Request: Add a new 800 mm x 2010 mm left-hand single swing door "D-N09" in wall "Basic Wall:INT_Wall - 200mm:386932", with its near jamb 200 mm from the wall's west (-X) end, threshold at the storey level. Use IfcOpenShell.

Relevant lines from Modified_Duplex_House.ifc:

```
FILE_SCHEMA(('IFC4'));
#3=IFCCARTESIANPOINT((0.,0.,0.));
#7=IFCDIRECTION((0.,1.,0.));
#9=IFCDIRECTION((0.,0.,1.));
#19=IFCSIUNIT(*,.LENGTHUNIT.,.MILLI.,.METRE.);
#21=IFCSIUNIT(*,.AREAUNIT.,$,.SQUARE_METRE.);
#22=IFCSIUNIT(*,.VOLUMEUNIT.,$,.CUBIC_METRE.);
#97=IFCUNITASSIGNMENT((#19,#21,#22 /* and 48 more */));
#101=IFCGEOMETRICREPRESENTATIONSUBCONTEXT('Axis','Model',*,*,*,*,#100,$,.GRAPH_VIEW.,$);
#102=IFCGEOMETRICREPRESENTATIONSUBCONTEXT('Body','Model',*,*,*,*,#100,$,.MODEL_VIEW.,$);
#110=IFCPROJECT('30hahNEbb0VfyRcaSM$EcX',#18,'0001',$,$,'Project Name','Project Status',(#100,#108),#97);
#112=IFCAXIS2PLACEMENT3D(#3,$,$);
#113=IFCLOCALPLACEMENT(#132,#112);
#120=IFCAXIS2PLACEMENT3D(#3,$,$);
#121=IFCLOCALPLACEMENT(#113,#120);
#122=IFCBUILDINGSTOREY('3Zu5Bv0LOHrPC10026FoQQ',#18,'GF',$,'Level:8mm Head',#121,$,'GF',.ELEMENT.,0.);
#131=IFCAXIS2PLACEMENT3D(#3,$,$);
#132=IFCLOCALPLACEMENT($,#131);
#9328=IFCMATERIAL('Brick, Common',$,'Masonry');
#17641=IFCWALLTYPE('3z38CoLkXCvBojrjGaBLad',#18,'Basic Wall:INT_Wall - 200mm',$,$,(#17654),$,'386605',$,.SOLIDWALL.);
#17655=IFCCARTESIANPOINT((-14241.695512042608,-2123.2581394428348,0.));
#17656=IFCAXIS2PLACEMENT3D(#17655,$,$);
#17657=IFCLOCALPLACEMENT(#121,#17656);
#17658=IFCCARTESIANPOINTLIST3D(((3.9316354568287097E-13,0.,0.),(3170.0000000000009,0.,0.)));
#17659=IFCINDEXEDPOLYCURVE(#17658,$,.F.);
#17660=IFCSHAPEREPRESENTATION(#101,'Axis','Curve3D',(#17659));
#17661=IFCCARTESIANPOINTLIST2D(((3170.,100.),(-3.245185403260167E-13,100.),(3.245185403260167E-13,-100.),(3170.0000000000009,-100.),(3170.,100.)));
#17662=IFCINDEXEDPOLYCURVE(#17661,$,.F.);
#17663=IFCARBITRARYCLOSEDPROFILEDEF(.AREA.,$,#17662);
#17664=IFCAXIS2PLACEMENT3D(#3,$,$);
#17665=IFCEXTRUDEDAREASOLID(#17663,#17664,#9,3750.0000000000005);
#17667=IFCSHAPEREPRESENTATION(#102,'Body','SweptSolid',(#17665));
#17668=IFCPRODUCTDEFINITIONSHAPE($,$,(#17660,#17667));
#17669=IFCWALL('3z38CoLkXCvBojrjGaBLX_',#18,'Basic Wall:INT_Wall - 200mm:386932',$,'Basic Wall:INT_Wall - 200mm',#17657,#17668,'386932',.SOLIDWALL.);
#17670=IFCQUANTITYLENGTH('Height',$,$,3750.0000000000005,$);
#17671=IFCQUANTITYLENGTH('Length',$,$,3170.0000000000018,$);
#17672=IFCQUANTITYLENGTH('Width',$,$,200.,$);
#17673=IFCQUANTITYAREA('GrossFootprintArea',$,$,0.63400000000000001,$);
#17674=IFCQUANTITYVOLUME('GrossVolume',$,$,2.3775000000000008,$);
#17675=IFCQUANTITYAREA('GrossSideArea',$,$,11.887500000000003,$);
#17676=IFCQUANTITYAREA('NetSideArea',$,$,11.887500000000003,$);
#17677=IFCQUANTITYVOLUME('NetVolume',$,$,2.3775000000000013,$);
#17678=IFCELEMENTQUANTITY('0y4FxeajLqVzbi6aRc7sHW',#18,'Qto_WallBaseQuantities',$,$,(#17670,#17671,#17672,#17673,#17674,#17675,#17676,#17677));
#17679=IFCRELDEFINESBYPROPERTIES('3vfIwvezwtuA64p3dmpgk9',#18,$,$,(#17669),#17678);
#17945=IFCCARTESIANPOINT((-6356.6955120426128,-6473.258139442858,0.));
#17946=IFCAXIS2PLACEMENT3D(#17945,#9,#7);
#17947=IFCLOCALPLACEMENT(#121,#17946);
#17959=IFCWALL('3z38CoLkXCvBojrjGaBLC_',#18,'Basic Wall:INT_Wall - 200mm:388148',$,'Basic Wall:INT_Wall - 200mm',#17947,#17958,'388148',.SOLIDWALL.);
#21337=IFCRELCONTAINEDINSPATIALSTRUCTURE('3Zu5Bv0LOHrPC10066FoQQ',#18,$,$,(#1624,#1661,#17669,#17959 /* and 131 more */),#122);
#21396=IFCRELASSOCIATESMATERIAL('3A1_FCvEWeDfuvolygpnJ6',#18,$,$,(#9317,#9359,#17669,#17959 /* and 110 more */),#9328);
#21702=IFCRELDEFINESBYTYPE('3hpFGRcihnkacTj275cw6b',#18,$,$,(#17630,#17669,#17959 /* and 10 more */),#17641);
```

```python
import numpy as np
import ifcopenshell
import ifcopenshell.api.feature
import ifcopenshell.api.geometry
import ifcopenshell.api.pset
import ifcopenshell.api.root
import ifcopenshell.api.spatial
import ifcopenshell.geom
import ifcopenshell.util.element
import ifcopenshell.util.placement
import ifcopenshell.util.representation
import ifcopenshell.util.shape
import ifcopenshell.util.unit

model = ifcopenshell.open("Modified_Duplex_House.ifc")
unit_scale = ifcopenshell.util.unit.calculate_unit_scale(model)
area_scale = ifcopenshell.util.unit.calculate_unit_scale(model, "AREAUNIT")
volume_scale = ifcopenshell.util.unit.calculate_unit_scale(model, "VOLUMEUNIT")
settings = ifcopenshell.geom.settings()


def volume(element):
    """Net volume in cubic metres, openings subtracted."""
    shape = ifcopenshell.geom.create_shape(settings, element)
    return ifcopenshell.util.shape.get_volume(shape.geometry)


wall = model.by_guid("3z38CoLkXCvBojrjGaBLX_")
storey = ifcopenshell.util.element.get_container(wall, ifc_class="IfcBuildingStorey")
context = ifcopenshell.util.representation.get_context(model, "Model", "Body", "MODEL_VIEW")
before = volume(wall)

width, height, from_end, sill = 0.8, 2.01, 0.2, 0.0  # metres

# The wall runs along its own X axis, and the end named is its -X end.
wall_shape = ifcopenshell.geom.create_shape(settings, wall)
x, y, z = ifcopenshell.util.shape.get_vertices(wall_shape.geometry).T
start = x.min() + from_end
face, thickness = float(y.min()), float(y.max() - y.min())
wall_matrix = ifcopenshell.util.placement.get_local_placement(wall.ObjectPlacement)
level = ifcopenshell.util.placement.get_local_placement(storey.ObjectPlacement)[2, 3]


def in_wall(x, y):
    """Placement at x, y metres in the wall's axes, at sill height."""
    matrix = wall_matrix.copy()
    matrix[:, 3] = wall_matrix @ np.array([x / unit_scale, y / unit_scale, 0.0, 1.0])
    matrix[2, 3] = level + sill / unit_scale
    return matrix


# Opening: a box that overshoots both wall faces by 50 mm.
opening = ifcopenshell.api.root.create_entity(model, ifc_class="IfcOpeningElement", predefined_type="OPENING")
box = ifcopenshell.api.geometry.add_wall_representation(
    model, context=context, length=width, height=height, thickness=thickness + 0.1
)
ifcopenshell.api.geometry.assign_representation(model, product=opening, representation=box)
ifcopenshell.api.geometry.edit_object_placement(model, product=opening, matrix=in_wall(start, face - 0.05), is_si=False)
ifcopenshell.api.feature.add_feature(model, feature=opening, element=wall)

door = ifcopenshell.api.root.create_entity(model, ifc_class="IfcDoor", name="D-N09", predefined_type="DOOR")
door.OverallWidth, door.OverallHeight = width / unit_scale, height / unit_scale
door.OperationType = "SINGLE_SWING_LEFT"
body = ifcopenshell.api.geometry.add_door_representation(
    model,
    context=context,
    overall_width=door.OverallWidth,
    overall_height=door.OverallHeight,
    operation_type="SINGLE_SWING_LEFT",
    lining_properties={"LiningDepth": thickness / unit_scale, "ThresholdDepth": thickness / unit_scale},
)
ifcopenshell.api.geometry.assign_representation(model, product=door, representation=body)
ifcopenshell.api.spatial.assign_container(model, products=[door], relating_structure=storey)
ifcopenshell.api.feature.add_filling(model, opening=opening, element=door)

# The lining spans the wall, so the door starts at the wall face.
ifcopenshell.api.geometry.edit_object_placement(model, product=door, matrix=in_wall(start, face), is_si=False)

after = volume(wall)

# Update the wall's stored quantities.
qto = model.by_id(ifcopenshell.util.element.get_pset(wall, "Qto_WallBaseQuantities", should_inherit=False)["id"])
ifcopenshell.api.pset.edit_qto(model, qto=qto, properties={
    "NetSideArea": after / thickness / area_scale,
    "NetVolume": after / volume_scale,
})

print(f"wall volume {before:.3f} -> {after:.3f} m3")

model.write("Modified_Duplex_House_rev.ifc")
```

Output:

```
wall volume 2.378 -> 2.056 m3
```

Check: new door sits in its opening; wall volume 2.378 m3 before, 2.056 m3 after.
